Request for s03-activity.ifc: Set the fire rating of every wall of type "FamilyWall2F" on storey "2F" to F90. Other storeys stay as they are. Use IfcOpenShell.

First a look at what the model holds.

```python
import ifcopenshell
import ifcopenshell.util.element

model = ifcopenshell.open("s03-activity.ifc")
print(model.schema)
storey = next(s for s in model.by_type("IfcBuildingStorey") if s.Name == "2F")
walls = [e for e in ifcopenshell.util.element.get_decomposition(storey) if e.is_a("IfcWall")]
seen = {}
for e in walls:
    element_type = ifcopenshell.util.element.get_type(e)
    key = (element_type.Name if element_type != e and element_type else None, ifcopenshell.util.element.get_pset(e, "Pset_WallCommon", "FireRating"))
    seen[key] = seen.get(key, 0) + 1
for (name, value), count in sorted(seen.items(), key=str):
    print(count, "x", name, "|", value)
```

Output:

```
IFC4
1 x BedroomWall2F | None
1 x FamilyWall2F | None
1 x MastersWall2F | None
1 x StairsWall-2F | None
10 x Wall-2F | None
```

```python
import ifcopenshell
import ifcopenshell.api.pset
import ifcopenshell.util.element

model = ifcopenshell.open("s03-activity.ifc")

storey = next(s for s in model.by_type("IfcBuildingStorey") if s.Name == "2F")
walls = [e for e in ifcopenshell.util.element.get_decomposition(storey) if e.is_a("IfcWall")]

count = 0
for e in walls:
    element_type = ifcopenshell.util.element.get_type(e)
    if element_type in (None, e) or element_type.Name != "FamilyWall2F":
        continue
    # add_pset returns the element's existing set when there is one.
    pset = ifcopenshell.api.pset.add_pset(model, product=e, name="Pset_WallCommon")
    ifcopenshell.api.pset.edit_pset(model, pset=pset, properties={"FireRating": "F90"})
    count += 1

print(count, "walls updated")

model.write("s03-activity_edited.ifc")
```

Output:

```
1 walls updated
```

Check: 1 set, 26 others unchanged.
